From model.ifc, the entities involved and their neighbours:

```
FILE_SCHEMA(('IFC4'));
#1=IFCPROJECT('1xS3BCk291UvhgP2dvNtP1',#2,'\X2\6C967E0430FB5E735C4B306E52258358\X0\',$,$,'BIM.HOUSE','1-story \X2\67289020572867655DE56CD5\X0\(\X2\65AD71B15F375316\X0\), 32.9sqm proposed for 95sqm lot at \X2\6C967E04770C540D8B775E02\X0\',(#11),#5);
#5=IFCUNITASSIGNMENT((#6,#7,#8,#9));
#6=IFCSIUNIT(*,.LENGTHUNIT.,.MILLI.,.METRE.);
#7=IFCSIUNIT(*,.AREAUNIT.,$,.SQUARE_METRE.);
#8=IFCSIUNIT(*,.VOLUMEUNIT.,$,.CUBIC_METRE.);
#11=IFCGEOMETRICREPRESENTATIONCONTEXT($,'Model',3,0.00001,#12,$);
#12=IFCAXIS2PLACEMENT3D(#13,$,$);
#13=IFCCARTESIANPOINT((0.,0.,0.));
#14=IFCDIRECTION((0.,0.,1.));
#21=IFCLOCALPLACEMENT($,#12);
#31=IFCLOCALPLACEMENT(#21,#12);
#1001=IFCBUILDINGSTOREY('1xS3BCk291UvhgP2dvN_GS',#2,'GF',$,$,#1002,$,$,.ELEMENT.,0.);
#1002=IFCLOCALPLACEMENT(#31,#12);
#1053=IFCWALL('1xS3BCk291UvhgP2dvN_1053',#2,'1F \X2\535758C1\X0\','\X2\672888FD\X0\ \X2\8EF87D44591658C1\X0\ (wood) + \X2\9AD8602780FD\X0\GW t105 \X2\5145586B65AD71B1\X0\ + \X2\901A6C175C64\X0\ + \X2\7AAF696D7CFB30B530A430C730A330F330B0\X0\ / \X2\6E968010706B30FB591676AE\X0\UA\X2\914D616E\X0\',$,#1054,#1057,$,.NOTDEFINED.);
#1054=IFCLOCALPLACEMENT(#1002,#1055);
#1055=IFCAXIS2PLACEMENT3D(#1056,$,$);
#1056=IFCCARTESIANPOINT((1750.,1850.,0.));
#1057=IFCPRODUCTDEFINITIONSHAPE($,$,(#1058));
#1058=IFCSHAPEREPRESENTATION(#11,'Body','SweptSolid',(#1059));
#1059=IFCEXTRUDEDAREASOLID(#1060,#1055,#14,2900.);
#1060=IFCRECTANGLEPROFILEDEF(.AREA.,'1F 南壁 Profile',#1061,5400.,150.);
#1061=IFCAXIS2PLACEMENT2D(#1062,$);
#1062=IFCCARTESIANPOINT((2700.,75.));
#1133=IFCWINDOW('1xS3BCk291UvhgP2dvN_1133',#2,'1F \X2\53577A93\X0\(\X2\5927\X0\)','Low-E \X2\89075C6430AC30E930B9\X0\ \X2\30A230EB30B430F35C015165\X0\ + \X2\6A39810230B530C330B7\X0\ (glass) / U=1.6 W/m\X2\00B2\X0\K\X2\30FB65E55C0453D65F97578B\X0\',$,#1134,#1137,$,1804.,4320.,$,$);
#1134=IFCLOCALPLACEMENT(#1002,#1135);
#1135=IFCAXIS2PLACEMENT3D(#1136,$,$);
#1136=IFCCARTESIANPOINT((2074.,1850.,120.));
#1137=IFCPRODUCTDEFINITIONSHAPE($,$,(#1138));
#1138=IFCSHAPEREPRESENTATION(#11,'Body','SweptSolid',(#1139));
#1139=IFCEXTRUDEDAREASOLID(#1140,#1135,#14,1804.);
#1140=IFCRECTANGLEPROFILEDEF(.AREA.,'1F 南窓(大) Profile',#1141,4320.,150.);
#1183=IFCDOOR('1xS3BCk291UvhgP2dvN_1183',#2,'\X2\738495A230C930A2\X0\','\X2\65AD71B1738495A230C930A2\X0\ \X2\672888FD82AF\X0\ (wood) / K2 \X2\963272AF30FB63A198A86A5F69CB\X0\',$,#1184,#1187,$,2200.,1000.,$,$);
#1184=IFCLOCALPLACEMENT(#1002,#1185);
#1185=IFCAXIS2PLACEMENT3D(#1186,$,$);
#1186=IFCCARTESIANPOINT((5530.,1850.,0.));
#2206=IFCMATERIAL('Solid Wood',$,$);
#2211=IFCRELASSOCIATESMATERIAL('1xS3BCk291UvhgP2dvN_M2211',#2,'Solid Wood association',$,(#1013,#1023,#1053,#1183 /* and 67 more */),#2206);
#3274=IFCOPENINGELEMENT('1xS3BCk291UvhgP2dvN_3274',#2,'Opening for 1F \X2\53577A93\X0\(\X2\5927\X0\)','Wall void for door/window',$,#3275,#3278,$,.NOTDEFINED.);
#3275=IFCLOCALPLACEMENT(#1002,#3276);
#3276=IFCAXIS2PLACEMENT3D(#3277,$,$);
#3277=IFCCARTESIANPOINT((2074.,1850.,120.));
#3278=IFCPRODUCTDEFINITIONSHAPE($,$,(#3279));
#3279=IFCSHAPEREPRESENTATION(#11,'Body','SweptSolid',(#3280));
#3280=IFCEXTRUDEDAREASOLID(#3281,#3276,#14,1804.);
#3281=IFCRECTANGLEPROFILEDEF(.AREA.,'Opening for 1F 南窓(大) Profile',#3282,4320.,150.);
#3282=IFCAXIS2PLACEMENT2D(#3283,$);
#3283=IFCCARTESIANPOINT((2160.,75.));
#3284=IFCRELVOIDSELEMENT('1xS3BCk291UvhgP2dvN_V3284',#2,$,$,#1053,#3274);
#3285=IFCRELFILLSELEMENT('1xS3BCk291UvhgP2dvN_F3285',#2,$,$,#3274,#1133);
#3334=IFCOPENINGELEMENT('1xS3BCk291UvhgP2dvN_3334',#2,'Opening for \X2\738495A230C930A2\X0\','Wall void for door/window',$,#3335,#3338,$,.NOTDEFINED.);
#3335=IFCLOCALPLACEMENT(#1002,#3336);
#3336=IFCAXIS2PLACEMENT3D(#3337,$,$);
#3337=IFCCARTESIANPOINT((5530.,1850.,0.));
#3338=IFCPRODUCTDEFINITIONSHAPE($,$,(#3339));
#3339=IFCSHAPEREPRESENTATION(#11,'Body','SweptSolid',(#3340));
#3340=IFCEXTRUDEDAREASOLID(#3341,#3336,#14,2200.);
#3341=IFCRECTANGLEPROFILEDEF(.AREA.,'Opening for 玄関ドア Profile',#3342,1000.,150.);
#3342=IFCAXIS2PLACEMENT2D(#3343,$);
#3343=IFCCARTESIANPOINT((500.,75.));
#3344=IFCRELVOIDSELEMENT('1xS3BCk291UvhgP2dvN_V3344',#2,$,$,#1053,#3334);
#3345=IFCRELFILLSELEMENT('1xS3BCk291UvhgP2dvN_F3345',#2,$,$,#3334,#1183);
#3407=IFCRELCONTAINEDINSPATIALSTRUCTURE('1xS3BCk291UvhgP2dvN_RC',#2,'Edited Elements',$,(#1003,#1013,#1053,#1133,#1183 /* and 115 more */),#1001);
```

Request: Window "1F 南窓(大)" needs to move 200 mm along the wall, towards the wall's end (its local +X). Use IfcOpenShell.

```python
import ifcopenshell
import ifcopenshell.api.geometry
import ifcopenshell.util.placement
import ifcopenshell.util.unit

model = ifcopenshell.open("model.ifc")
unit_scale = ifcopenshell.util.unit.calculate_unit_scale(model)

window = model.by_id(1133)
opening = window.FillsVoids[0].RelatingOpeningElement
wall = opening.VoidsElements[0].RelatingBuildingElement

wall_matrix = ifcopenshell.util.placement.get_local_placement(wall.ObjectPlacement)
shift = wall_matrix[:3, 0] * 0.2 / unit_scale
before = ifcopenshell.util.placement.get_local_placement(window.ObjectPlacement)[:3, 3].copy()

# The window is not placed relative to its opening, so move both.
for product in (opening, window):
    matrix = ifcopenshell.util.placement.get_local_placement(product.ObjectPlacement)
    matrix[:3, 3] += shift
    ifcopenshell.api.geometry.edit_object_placement(model, product=product, matrix=matrix, is_si=False)

after = ifcopenshell.util.placement.get_local_placement(window.ObjectPlacement)[:3, 3]
print("window moved by", (after - before).round(3) + 0.0)

model.write("model_edited.ifc")
```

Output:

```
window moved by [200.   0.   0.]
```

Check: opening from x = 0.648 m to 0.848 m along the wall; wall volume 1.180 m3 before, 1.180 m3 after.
